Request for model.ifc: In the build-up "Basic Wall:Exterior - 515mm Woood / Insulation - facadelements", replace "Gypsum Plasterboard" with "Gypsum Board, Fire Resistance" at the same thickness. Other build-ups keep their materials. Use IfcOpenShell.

First a look at what the model holds.

```python
import ifcopenshell
import ifcopenshell.util.element

model = ifcopenshell.open("model.ifc")
print(model.schema)
for layer_set in model.by_type("IfcMaterialLayerSet"):
    if layer_set.LayerSetName == "Basic Wall:Exterior - 515mm Woood / Insulation - facadelements":
        for layer in layer_set.MaterialLayers:
            print(layer.id(), layer.Material and layer.Material.Name, layer.LayerThickness, sep=" | ")
        print(len(ifcopenshell.util.element.get_elements_by_material(model, layer_set)), "elements and types use it")
print(sorted(m.Name for m in model.by_type("IfcMaterial") if m.Name)[:60])
```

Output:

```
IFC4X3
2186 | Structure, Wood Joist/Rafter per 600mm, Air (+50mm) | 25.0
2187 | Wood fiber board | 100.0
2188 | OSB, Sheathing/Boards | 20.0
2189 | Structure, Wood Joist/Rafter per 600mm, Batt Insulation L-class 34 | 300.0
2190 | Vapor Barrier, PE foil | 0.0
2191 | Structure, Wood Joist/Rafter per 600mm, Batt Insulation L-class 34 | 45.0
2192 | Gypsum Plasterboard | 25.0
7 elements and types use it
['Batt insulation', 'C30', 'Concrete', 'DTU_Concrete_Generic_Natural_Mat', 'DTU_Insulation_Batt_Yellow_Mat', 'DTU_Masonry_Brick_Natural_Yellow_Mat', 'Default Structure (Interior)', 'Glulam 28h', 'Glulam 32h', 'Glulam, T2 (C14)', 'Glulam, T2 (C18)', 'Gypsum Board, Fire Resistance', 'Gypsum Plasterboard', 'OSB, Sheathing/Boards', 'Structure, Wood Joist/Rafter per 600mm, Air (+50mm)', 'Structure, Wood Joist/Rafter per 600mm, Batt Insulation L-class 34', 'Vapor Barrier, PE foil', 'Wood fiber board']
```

```python
import ifcopenshell
import ifcopenshell.api.material

model = ifcopenshell.open("model.ifc")

layer_set = next(s for s in model.by_type("IfcMaterialLayerSet") if s.LayerSetName == "Basic Wall:Exterior - 515mm Woood / Insulation - facadelements")
layer = next(l for l in layer_set.MaterialLayers if l.Material and l.Material.Name == "Gypsum Plasterboard")
material = next(m for m in model.by_type("IfcMaterial") if m.Name == "Gypsum Board, Fire Resistance")

# Point this one layer at the other material; renaming the old one would change it everywhere.
ifcopenshell.api.material.edit_layer(model, layer=layer, attributes={"Name": material.Name}, material=material)

print([l.Material.Name if l.Material else None for l in layer_set.MaterialLayers])

model.write("model_v2.ifc")
```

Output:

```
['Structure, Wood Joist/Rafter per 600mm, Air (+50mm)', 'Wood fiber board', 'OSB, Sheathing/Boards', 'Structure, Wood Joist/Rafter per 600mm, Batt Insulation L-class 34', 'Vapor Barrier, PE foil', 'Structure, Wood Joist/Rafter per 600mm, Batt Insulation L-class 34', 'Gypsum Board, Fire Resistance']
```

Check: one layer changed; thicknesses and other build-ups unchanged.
